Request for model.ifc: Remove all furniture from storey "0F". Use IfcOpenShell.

First a look at what the model holds.

```python
import ifcopenshell
import ifcopenshell.util.element

model = ifcopenshell.open("model.ifc")
print(model.schema)
storey = next(s for s in model.by_type("IfcBuildingStorey") if s.Name == "0F")
furniture = [e for e in ifcopenshell.util.element.get_decomposition(storey) if e.is_a("IfcFurnishingElement")]
seen = {}
for e in furniture:
    element_type = ifcopenshell.util.element.get_type(e)
    name = element_type.Name if element_type not in (None, e) else None
    seen[name] = seen.get(name, 0) + 1
for name, count in sorted(seen.items(), key=str):
    print(count, "x", name)
```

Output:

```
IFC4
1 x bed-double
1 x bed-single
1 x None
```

```python
import ifcopenshell
import ifcopenshell.api.root
import ifcopenshell.util.element

model = ifcopenshell.open("model.ifc")

storey = next(s for s in model.by_type("IfcBuildingStorey") if s.Name == "0F")
furniture = [e for e in ifcopenshell.util.element.get_decomposition(storey) if e.is_a("IfcFurnishingElement")]

for e in furniture:
    ifcopenshell.api.root.remove_product(model, product=e)
print(len(furniture), "removed")

model.write("model-out.ifc")
```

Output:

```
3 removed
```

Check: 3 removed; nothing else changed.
